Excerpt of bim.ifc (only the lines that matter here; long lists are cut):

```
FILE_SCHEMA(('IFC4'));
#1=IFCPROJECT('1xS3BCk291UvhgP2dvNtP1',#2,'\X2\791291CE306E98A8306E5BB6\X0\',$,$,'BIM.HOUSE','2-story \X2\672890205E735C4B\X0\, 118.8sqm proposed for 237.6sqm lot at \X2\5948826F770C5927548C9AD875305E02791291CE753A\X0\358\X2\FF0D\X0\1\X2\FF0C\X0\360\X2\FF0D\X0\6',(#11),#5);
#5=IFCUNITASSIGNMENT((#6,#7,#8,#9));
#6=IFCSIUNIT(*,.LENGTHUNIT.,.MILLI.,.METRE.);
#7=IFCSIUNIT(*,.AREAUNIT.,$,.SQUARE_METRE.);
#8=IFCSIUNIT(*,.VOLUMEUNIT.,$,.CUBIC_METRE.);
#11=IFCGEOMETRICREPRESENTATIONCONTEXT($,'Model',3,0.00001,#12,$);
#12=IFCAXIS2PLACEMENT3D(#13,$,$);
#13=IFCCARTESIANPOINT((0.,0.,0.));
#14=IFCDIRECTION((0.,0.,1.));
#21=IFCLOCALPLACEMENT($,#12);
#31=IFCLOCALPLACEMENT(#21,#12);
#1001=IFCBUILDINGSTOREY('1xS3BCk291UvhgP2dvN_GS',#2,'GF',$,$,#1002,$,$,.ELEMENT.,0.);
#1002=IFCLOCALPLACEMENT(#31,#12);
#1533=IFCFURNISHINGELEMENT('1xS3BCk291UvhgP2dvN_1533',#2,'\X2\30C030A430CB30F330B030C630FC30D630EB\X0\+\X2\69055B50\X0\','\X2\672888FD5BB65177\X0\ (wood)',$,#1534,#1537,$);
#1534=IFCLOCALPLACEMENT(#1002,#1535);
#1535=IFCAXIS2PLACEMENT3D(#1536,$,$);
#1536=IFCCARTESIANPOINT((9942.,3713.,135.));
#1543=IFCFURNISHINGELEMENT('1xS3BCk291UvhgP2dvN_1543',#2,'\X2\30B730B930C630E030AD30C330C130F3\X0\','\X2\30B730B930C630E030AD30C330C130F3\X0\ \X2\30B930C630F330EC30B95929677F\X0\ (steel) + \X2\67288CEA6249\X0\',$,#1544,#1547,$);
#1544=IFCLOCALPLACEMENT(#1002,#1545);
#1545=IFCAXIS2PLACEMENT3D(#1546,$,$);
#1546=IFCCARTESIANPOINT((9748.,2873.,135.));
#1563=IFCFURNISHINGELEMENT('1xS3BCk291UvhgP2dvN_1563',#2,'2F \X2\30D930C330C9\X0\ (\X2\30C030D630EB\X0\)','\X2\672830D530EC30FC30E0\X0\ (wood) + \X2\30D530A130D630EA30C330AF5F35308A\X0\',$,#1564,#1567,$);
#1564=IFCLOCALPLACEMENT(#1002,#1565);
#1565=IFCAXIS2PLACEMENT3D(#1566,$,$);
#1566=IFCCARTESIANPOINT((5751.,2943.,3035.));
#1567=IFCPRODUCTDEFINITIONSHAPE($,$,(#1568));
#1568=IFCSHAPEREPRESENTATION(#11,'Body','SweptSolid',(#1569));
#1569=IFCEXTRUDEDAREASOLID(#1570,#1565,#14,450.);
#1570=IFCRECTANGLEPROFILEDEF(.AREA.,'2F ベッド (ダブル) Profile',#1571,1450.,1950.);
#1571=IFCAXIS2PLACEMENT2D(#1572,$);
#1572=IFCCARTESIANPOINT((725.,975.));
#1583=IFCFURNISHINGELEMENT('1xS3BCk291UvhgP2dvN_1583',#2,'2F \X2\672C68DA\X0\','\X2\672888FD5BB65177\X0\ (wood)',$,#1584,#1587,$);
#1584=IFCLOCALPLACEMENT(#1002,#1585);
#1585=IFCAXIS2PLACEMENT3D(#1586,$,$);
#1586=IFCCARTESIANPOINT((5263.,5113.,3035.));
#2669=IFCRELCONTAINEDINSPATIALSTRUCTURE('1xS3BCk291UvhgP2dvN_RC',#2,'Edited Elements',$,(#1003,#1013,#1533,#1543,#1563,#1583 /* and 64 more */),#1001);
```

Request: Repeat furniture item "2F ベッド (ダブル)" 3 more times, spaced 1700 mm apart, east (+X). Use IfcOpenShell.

```python
import numpy as np
import ifcopenshell
import ifcopenshell.api.geometry
import ifcopenshell.api.root
import ifcopenshell.util.element
import ifcopenshell.util.placement
import ifcopenshell.util.unit

model = ifcopenshell.open("bim.ifc")
unit_scale = ifcopenshell.util.unit.calculate_unit_scale(model)


def reuse_history(source, copy):
    """copy_class also copies each property set's owner history, people and application; keep the originals."""
    for rel in copy.IsDefinedBy:
        if rel.is_a("IfcRelDefinesByProperties") and (history := rel.RelatingPropertyDefinition.OwnerHistory):
            rel.RelatingPropertyDefinition.OwnerHistory = source.OwnerHistory
            ifcopenshell.util.element.remove_deep2(model, history)


source = model.by_guid("1xS3BCk291UvhgP2dvN_1563")
base = ifcopenshell.util.placement.get_local_placement(source.ObjectPlacement)
step = np.array([1.0, 0.0, 0.0]) * 1.7 / unit_scale

for i in range(1, 4):
    copy = ifcopenshell.api.root.copy_class(model, product=source)
    copy.Representation = ifcopenshell.util.element.copy_deep(
        model, source.Representation, exclude=["IfcGeometricRepresentationContext", "IfcRepresentationMap"]
    )
    reuse_history(source, copy)
    matrix = base.copy()
    matrix[:3, 3] += i * step
    print("added at", matrix[:3, 3].round(3) + 0.0)
    ifcopenshell.api.geometry.edit_object_placement(model, product=copy, matrix=matrix, is_si=False)

model.write("bim_v2.ifc")
```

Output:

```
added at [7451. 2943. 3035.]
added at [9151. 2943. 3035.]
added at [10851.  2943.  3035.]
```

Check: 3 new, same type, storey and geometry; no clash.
